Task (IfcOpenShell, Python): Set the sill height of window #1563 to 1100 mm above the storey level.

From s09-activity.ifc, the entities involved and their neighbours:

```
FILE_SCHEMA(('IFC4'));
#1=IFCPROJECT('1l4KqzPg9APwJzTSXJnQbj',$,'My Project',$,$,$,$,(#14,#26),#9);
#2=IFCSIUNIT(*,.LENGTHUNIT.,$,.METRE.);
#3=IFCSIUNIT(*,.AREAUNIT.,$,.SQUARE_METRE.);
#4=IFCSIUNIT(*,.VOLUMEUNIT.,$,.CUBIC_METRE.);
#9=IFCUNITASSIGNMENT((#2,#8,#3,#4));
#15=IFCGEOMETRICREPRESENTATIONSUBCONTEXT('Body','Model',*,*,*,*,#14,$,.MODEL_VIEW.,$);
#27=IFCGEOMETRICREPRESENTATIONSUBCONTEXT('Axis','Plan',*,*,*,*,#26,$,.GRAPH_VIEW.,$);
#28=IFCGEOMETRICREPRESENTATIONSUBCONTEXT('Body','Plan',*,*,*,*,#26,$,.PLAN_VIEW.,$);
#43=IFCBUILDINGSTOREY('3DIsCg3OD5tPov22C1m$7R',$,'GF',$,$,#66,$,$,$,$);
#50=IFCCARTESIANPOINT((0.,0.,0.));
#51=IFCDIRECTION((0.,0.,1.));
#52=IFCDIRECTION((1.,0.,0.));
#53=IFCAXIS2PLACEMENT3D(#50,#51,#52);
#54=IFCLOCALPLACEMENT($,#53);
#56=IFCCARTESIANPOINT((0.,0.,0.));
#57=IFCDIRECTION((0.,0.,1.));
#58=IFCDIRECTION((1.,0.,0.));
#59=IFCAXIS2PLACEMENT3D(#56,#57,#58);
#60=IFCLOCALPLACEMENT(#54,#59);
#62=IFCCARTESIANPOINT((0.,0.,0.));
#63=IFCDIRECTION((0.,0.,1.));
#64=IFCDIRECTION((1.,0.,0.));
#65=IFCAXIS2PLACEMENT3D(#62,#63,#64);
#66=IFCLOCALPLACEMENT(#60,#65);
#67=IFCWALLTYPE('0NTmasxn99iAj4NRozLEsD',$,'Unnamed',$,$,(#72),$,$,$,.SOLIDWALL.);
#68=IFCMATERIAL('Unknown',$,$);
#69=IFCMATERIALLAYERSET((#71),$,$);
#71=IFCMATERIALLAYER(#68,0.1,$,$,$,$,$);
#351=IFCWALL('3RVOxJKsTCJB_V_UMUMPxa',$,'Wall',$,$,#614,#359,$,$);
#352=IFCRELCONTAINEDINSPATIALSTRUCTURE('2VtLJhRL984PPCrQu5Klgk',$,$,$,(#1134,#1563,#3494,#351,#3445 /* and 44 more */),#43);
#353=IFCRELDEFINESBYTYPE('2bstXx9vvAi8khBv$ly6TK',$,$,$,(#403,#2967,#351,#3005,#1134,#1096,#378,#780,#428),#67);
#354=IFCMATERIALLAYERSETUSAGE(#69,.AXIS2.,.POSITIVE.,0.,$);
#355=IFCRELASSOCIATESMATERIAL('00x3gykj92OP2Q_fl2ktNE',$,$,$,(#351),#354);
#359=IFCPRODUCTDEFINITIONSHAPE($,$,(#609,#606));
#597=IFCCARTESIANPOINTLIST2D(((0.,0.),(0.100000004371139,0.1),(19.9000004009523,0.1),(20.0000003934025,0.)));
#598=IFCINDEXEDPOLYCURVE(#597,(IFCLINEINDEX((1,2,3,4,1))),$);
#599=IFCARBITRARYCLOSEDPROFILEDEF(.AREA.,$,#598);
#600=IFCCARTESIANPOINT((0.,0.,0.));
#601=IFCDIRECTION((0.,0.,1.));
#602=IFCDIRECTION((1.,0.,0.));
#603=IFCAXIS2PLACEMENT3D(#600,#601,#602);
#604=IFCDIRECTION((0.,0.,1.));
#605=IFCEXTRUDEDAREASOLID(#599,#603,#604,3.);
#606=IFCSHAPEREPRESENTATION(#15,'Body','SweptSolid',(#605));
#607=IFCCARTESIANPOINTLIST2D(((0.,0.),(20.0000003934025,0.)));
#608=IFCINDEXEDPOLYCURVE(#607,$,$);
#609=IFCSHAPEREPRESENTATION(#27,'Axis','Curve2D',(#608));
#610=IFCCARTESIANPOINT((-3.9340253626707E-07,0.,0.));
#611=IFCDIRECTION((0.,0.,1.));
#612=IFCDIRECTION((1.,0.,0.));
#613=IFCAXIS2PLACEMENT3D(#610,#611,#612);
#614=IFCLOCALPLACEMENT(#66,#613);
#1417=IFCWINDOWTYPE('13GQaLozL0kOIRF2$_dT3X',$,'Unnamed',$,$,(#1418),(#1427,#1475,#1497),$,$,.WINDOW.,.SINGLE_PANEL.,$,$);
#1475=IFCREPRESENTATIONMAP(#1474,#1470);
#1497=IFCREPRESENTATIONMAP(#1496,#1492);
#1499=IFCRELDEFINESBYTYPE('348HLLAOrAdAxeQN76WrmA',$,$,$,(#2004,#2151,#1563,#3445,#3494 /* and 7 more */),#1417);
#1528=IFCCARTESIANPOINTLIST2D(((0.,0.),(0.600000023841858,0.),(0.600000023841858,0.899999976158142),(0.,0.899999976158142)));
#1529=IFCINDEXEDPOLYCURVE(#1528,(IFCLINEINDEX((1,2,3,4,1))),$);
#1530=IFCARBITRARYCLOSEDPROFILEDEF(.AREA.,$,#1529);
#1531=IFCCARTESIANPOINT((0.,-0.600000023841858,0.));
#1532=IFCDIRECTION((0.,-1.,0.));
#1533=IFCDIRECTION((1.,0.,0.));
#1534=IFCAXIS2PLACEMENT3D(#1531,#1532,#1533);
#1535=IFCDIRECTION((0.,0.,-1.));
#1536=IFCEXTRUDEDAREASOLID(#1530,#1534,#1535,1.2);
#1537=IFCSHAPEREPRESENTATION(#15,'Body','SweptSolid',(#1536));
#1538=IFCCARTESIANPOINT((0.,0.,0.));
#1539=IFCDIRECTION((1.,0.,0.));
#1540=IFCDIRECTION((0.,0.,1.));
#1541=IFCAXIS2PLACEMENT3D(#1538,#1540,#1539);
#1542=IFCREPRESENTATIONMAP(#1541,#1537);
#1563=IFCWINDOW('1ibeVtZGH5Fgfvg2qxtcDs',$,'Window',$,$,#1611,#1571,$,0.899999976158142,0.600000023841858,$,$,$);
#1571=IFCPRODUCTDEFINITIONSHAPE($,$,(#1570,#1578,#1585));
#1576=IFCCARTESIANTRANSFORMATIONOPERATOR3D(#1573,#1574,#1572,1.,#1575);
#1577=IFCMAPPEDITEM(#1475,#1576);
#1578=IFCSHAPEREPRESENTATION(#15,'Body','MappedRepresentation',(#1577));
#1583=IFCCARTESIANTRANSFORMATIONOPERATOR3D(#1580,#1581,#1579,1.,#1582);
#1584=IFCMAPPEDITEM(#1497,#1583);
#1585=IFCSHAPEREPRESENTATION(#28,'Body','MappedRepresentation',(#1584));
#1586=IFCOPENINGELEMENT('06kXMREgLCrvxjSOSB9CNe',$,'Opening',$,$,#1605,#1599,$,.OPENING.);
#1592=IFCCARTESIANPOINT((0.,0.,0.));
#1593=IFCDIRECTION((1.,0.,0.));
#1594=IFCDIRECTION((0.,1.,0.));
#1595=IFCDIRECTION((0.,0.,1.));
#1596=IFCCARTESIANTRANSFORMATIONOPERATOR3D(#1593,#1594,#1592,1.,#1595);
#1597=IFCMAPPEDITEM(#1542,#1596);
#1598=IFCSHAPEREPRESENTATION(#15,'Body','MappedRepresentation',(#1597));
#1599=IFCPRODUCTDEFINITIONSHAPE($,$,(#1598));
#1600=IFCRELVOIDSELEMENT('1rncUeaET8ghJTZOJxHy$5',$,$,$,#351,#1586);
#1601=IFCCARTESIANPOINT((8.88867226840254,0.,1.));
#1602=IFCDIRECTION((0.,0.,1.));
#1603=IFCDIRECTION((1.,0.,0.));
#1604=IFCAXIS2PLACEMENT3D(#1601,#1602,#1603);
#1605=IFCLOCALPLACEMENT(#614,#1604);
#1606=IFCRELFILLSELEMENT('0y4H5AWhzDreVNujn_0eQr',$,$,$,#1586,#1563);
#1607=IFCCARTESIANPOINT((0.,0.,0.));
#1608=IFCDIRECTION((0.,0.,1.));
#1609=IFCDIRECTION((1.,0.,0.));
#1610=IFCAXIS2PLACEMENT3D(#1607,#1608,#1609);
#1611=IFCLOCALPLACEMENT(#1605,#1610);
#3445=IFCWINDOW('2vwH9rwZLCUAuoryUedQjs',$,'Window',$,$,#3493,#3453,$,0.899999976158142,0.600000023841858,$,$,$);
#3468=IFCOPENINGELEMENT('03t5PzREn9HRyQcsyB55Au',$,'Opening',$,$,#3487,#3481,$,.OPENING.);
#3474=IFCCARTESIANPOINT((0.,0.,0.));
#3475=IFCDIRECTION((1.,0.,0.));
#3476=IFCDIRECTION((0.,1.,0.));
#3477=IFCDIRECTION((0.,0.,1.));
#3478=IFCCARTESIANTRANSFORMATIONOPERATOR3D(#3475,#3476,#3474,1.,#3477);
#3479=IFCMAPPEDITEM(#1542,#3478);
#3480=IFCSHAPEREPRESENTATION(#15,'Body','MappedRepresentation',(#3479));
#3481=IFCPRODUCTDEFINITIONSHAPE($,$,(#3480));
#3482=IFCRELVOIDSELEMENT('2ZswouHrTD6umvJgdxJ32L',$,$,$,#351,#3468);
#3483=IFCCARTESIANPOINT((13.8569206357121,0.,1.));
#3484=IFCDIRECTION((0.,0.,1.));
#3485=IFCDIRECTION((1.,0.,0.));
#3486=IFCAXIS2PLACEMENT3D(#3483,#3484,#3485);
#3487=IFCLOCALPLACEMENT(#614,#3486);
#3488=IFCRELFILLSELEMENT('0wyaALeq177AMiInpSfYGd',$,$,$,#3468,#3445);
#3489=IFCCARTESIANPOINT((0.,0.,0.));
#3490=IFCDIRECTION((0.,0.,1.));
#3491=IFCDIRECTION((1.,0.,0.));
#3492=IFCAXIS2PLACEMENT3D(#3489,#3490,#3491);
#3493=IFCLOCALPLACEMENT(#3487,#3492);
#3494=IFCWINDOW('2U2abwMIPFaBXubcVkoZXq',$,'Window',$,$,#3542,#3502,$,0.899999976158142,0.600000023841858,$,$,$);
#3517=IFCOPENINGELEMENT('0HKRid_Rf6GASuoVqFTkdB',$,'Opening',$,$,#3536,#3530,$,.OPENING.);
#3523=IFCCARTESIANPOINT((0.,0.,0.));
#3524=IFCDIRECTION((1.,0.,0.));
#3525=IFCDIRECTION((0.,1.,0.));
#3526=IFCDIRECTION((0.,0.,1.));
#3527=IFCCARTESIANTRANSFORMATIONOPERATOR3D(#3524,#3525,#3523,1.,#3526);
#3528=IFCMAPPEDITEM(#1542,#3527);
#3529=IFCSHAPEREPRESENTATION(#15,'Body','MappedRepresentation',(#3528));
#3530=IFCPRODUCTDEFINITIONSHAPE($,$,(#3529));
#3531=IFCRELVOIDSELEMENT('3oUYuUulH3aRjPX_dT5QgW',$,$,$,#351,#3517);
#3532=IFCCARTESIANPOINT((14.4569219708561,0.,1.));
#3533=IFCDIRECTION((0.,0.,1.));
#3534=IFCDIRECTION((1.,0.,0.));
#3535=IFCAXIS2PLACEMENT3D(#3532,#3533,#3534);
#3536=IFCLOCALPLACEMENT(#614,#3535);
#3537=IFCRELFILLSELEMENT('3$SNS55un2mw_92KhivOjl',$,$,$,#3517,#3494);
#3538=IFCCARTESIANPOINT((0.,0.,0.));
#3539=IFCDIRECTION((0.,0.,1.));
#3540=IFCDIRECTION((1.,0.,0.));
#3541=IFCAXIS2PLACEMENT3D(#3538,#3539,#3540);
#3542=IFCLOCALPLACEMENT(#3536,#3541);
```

```python
import numpy as np
import ifcopenshell
import ifcopenshell.api.geometry
import ifcopenshell.geom
import ifcopenshell.util.element
import ifcopenshell.util.placement
import ifcopenshell.util.shape
import ifcopenshell.util.unit

model = ifcopenshell.open("s09-activity.ifc")
unit_scale = ifcopenshell.util.unit.calculate_unit_scale(model)

window = model.by_guid("1ibeVtZGH5Fgfvg2qxtcDs")
opening = window.FillsVoids[0].RelatingOpeningElement
storey = ifcopenshell.util.element.get_container(window, ifc_class="IfcBuildingStorey")
level = ifcopenshell.util.placement.get_local_placement(storey.ObjectPlacement)[2, 3]

# The opening's origin need not be at the sill, so measure its lowest point.
shape = ifcopenshell.geom.create_shape(ifcopenshell.geom.settings(), opening)
bottom = ifcopenshell.util.shape.get_shape_bottom_elevation(shape, shape.geometry) / unit_scale
dz = level + 1.1 / unit_scale - bottom

shift = np.array([0.0, 0.0, dz])
# The window is placed relative to its opening, so it follows when the opening moves.
matrix = ifcopenshell.util.placement.get_local_placement(opening.ObjectPlacement)
matrix[:3, 3] += shift
ifcopenshell.api.geometry.edit_object_placement(
    model, product=opening, matrix=matrix, is_si=False, should_transform_children=True
)

print(f"moved by {dz * unit_scale:+.3f} m")

model.write("s09-activity-out.ifc")
```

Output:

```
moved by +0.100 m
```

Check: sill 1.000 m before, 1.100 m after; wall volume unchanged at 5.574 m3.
